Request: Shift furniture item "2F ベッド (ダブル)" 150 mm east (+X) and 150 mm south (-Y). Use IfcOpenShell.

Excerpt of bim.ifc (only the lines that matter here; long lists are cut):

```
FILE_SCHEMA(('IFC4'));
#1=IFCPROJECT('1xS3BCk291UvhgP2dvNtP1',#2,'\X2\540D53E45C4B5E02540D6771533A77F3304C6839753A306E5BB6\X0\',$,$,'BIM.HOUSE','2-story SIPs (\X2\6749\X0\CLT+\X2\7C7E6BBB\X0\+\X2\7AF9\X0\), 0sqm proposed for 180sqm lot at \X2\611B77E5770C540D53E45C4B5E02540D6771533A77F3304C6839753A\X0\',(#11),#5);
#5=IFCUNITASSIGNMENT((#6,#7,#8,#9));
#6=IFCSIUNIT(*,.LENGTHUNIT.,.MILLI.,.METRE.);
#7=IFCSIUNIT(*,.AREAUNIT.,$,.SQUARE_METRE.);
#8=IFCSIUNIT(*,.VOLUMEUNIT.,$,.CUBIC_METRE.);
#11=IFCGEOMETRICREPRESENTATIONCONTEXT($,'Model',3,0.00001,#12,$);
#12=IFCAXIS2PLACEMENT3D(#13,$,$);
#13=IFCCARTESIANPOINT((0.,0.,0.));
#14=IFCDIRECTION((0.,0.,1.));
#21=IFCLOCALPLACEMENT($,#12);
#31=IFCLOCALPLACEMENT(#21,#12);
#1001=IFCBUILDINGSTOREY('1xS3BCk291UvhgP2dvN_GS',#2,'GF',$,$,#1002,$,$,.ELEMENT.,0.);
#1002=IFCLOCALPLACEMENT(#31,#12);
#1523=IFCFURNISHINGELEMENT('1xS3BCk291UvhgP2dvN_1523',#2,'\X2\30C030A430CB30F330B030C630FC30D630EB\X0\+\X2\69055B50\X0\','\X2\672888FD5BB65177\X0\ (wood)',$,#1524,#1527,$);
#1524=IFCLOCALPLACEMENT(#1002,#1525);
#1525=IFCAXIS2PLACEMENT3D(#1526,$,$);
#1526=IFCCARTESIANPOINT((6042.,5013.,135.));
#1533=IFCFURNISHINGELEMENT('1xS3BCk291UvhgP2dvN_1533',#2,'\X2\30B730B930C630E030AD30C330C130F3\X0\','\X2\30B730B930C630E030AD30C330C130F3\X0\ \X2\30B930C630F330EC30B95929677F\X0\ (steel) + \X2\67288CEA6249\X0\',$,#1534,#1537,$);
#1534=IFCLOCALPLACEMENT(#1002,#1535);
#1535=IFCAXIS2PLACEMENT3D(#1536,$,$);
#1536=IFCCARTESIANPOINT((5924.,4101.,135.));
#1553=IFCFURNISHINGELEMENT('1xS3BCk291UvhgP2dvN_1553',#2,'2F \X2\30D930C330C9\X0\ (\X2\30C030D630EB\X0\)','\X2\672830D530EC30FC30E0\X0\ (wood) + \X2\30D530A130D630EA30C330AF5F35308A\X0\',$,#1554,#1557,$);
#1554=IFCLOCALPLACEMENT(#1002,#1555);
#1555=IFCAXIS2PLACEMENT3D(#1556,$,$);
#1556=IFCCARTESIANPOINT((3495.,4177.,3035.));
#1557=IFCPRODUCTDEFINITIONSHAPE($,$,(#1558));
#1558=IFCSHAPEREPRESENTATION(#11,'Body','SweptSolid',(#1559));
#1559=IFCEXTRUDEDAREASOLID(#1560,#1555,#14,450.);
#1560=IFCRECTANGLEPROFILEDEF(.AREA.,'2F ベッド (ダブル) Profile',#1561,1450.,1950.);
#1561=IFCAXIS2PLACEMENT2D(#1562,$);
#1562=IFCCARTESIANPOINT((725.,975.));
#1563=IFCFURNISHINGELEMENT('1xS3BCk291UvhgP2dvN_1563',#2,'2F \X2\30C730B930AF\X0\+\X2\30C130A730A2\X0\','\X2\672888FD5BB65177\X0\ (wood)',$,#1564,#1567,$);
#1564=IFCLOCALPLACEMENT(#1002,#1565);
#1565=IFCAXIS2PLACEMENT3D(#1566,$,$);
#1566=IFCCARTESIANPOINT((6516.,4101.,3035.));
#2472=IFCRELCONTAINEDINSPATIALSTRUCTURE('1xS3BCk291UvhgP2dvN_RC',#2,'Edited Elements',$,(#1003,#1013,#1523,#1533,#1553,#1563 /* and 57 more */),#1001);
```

```python
import ifcopenshell
import ifcopenshell.api.geometry
import ifcopenshell.util.placement
import ifcopenshell.util.unit

model = ifcopenshell.open("bim.ifc")
unit_scale = ifcopenshell.util.unit.calculate_unit_scale(model)

item = model.by_guid("1xS3BCk291UvhgP2dvN_1553")
matrix = ifcopenshell.util.placement.get_local_placement(item.ObjectPlacement)
matrix[0, 3] += 0.15 / unit_scale
matrix[1, 3] -= 0.15 / unit_scale
ifcopenshell.api.geometry.edit_object_placement(model, product=item, matrix=matrix, is_si=False)

print(ifcopenshell.util.placement.get_local_placement(item.ObjectPlacement).round(3) + 0.0)

model.write("bim-out.ifc")
```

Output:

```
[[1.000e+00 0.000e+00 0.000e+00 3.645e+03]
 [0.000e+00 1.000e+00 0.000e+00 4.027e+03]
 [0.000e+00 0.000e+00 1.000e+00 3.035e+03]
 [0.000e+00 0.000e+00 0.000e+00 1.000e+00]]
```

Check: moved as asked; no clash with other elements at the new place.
